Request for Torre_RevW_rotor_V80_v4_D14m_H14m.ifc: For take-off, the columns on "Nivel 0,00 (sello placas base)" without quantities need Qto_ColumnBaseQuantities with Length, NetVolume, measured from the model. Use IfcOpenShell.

First a look at what the model holds.

```python
import ifcopenshell
import ifcopenshell.util.element
import ifcopenshell.util.unit

model = ifcopenshell.open("Torre_RevW_rotor_V80_v4_D14m_H14m.ifc")
print(model.schema)
for unit_type in ("LENGTHUNIT", "AREAUNIT", "VOLUMEUNIT"):
    print(unit_type, ifcopenshell.util.unit.calculate_unit_scale(model, unit_type))
storey = next(s for s in model.by_type("IfcBuildingStorey") if s.Name == "Nivel 0,00 (sello placas base)")
columns = [e for e in ifcopenshell.util.element.get_decomposition(storey) if e.is_a("IfcColumn")]
for e in sorted(columns, key=lambda e: e.id()):
    print(e.id(), e.is_a(), e.Name, list(ifcopenshell.util.element.get_psets(e, qtos_only=True)), sep=" | ")
```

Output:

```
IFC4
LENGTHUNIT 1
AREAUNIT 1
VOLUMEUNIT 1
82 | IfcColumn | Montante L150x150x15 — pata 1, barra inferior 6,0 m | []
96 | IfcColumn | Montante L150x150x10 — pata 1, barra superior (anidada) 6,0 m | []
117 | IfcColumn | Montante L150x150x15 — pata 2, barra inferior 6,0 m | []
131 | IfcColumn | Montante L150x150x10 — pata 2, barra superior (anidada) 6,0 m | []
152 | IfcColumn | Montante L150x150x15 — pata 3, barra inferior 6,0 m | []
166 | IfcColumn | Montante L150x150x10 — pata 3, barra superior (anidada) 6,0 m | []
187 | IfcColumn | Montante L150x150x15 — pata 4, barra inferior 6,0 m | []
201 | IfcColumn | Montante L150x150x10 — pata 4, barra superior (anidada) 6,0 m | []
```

```python
import ifcopenshell
import ifcopenshell.api.pset
import ifcopenshell.geom
import ifcopenshell.util.element
import ifcopenshell.util.shape
import ifcopenshell.util.unit

model = ifcopenshell.open("Torre_RevW_rotor_V80_v4_D14m_H14m.ifc")
unit_scale = ifcopenshell.util.unit.calculate_unit_scale(model)
volume_scale = ifcopenshell.util.unit.calculate_unit_scale(model, "VOLUMEUNIT")
settings = ifcopenshell.geom.settings()

storey = next(s for s in model.by_type("IfcBuildingStorey") if s.Name == "Nivel 0,00 (sello placas base)")
columns = [e for e in ifcopenshell.util.element.get_decomposition(storey) if e.is_a("IfcColumn")]

for e in sorted(columns, key=lambda e: e.id()):
    if ifcopenshell.util.element.get_psets(e, qtos_only=True, should_inherit=False):
        continue
    # Geometry comes back in metres, in the element's own axes.
    shape = ifcopenshell.geom.create_shape(settings, e)
    values = {
        "Length": ifcopenshell.util.shape.get_z(shape.geometry) / unit_scale,
        "NetVolume": ifcopenshell.util.shape.get_volume(shape.geometry) / volume_scale,
    }
    qto = ifcopenshell.api.pset.add_qto(model, product=e, name="Qto_ColumnBaseQuantities")
    ifcopenshell.api.pset.edit_qto(model, qto=qto, properties=values)
    print(e.id(), {k: round(v, 3) for k, v in values.items()})

model.write("Torre_RevW_rotor_V80_v4_D14m_H14m_updated.ifc")
```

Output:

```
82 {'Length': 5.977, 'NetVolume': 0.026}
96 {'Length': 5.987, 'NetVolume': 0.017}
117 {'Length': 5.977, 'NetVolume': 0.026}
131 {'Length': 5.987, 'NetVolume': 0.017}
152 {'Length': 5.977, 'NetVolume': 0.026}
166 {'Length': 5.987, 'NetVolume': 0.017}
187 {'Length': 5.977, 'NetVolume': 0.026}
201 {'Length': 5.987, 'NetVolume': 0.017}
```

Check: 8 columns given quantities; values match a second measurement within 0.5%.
